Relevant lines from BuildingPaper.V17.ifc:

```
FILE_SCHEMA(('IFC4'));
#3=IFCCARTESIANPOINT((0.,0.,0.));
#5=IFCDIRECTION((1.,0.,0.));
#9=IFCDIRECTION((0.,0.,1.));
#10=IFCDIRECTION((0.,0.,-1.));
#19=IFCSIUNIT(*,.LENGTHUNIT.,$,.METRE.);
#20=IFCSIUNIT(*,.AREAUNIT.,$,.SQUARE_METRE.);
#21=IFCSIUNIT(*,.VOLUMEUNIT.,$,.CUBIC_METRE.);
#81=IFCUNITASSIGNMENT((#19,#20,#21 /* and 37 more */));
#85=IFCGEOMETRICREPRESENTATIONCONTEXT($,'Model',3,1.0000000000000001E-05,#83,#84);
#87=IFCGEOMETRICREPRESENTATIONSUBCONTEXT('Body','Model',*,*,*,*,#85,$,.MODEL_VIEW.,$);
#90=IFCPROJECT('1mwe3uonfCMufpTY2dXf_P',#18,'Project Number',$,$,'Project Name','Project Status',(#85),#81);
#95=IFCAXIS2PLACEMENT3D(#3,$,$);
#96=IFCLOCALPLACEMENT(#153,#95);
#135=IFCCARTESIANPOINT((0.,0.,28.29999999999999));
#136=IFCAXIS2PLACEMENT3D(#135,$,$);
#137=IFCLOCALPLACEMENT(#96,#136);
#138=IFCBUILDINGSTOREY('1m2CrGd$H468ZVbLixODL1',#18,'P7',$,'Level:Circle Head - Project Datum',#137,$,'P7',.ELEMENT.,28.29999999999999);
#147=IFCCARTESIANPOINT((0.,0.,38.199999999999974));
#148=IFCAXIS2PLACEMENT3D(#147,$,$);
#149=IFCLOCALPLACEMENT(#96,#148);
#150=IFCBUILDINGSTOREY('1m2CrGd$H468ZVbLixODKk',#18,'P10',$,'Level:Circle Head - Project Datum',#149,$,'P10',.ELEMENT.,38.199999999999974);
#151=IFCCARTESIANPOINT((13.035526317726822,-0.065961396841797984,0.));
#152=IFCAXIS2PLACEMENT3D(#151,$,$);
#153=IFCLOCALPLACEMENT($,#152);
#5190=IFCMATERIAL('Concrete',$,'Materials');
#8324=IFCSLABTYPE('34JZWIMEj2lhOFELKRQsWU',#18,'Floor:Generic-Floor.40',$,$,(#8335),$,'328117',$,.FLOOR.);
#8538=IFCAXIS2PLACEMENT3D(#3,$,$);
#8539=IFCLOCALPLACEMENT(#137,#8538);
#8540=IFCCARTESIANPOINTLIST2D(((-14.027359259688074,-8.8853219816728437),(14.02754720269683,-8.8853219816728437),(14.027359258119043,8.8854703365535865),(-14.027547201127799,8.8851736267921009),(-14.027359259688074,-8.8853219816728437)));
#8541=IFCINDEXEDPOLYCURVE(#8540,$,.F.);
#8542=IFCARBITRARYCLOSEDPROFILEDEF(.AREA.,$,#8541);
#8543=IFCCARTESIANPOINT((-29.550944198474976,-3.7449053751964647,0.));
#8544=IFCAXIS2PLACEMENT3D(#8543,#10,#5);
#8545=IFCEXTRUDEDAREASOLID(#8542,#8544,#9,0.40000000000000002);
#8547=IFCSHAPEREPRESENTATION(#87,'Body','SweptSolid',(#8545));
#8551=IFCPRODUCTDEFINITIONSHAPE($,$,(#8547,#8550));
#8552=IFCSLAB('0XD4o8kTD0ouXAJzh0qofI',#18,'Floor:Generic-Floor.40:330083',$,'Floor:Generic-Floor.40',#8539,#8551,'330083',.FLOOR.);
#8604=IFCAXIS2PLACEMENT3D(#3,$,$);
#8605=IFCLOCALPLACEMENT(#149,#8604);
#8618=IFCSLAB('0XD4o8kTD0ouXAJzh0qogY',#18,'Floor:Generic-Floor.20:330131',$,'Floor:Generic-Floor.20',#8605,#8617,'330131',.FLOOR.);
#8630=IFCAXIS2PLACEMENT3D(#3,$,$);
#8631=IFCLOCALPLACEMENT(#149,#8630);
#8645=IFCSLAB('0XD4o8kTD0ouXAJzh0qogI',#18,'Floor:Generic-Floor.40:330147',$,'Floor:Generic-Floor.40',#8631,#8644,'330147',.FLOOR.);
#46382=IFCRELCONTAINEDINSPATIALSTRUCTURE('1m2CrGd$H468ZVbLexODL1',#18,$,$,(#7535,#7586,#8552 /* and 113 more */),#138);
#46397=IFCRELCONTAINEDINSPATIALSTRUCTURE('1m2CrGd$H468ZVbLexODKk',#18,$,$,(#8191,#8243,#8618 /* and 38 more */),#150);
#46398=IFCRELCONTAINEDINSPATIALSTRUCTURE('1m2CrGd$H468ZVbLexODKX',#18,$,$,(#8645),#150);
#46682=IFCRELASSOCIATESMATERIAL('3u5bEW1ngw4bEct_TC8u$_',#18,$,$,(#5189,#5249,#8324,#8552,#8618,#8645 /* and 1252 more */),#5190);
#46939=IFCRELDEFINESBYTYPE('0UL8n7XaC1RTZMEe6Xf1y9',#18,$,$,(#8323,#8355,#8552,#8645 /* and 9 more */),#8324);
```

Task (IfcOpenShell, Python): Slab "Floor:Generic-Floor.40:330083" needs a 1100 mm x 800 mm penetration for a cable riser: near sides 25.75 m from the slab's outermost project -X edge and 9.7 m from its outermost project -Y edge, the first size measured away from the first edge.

```python
import numpy as np
import ifcopenshell
import ifcopenshell.api.feature
import ifcopenshell.api.geometry
import ifcopenshell.api.root
import ifcopenshell.geom
import ifcopenshell.util.placement
import ifcopenshell.util.representation
import ifcopenshell.util.shape
import ifcopenshell.util.unit

model = ifcopenshell.open("BuildingPaper.V17.ifc")
unit_scale = ifcopenshell.util.unit.calculate_unit_scale(model)
settings = ifcopenshell.geom.settings()


def volume(element):
    """Net volume in cubic metres, openings subtracted."""
    shape = ifcopenshell.geom.create_shape(settings, element)
    return ifcopenshell.util.shape.get_volume(shape.geometry)


slab = model.by_guid("0XD4o8kTD0ouXAJzh0qofI")
before = volume(slab)

# Extent in the slab's own axes, in metres. The edges named are its -X and -Y sides.
slab_shape = ifcopenshell.geom.create_shape(settings, slab)
vertices = ifcopenshell.util.shape.get_vertices(slab_shape.geometry)
x_min, y_min, bottom = vertices.min(axis=0)
top = vertices[:, 2].max()

opening = ifcopenshell.api.root.create_entity(model, ifc_class="IfcOpeningElement", name="Cable riser opening", predefined_type="OPENING")
context = ifcopenshell.util.representation.get_context(model, "Model", "Body", "MODEL_VIEW")
width, depth = 1.1, 0.8
outline = [(0.0, 0.0), (width, 0.0), (width, depth), (0.0, depth), (0.0, 0.0)]
# Overshoot both faces by 50 mm so the cut is clean.
shape = ifcopenshell.api.geometry.add_slab_representation(
    model, context=context, depth=top - bottom + 0.1, polyline=outline
)
ifcopenshell.api.geometry.assign_representation(model, product=opening, representation=shape)

matrix = ifcopenshell.util.placement.get_local_placement(slab.ObjectPlacement)
matrix[:, 3] = matrix @ np.append(np.array([x_min + 25.75, y_min + 9.7, bottom - 0.05]) / unit_scale, 1.0)
ifcopenshell.api.geometry.edit_object_placement(model, product=opening, matrix=matrix, is_si=False)
ifcopenshell.api.feature.add_feature(model, feature=opening, element=slab)

after = volume(slab)

print(f"slab volume {before:.3f} -> {after:.3f} m3")

model.write("BuildingPaper.V17_rev.ifc")
```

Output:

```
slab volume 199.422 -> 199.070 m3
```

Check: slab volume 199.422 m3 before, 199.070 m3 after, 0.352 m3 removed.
